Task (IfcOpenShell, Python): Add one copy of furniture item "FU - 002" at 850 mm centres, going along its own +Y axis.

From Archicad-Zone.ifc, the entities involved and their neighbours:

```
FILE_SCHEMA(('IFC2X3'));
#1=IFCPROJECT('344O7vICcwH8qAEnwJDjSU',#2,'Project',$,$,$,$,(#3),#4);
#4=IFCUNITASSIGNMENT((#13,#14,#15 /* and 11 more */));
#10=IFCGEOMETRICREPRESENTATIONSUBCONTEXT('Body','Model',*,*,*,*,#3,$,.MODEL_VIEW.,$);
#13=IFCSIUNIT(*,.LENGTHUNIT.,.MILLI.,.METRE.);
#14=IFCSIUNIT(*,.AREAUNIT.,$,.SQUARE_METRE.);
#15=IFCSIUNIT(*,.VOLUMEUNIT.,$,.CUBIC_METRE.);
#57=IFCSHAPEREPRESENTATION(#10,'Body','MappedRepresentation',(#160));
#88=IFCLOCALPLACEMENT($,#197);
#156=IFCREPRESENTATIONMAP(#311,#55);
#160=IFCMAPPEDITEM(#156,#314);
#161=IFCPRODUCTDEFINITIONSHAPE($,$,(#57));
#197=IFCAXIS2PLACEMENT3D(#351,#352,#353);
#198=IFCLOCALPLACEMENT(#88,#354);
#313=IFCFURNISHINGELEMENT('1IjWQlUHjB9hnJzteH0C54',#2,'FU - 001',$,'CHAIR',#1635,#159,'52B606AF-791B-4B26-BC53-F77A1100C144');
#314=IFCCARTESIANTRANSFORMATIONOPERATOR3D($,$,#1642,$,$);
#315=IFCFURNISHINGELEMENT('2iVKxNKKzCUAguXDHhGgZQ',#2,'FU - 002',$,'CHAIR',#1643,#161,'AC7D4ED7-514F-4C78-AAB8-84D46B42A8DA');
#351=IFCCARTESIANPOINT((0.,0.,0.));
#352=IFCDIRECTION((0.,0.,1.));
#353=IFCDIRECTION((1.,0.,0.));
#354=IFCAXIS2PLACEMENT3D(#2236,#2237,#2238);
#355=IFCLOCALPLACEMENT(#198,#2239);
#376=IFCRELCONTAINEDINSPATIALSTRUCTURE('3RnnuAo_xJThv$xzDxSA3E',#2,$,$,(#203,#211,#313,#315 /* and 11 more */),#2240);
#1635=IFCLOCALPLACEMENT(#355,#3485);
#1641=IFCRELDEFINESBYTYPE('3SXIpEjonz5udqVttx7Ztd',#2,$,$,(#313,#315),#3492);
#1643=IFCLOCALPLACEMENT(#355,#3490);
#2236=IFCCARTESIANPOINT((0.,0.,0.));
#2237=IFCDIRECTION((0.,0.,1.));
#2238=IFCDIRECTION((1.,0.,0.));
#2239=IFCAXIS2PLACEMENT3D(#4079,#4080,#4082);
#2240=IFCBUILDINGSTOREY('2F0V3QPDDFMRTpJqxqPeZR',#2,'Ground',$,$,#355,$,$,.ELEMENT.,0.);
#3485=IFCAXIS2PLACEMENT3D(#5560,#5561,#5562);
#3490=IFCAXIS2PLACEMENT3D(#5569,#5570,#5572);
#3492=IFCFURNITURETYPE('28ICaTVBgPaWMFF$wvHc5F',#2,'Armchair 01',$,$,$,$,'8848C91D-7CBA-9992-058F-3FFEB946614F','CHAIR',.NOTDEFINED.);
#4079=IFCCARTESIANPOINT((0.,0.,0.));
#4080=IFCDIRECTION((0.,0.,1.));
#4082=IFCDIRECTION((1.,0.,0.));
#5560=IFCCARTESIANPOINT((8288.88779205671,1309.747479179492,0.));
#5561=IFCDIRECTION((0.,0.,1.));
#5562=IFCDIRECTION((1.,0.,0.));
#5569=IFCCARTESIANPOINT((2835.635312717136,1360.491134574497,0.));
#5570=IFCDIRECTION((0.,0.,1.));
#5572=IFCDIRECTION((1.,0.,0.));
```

```python
import ifcopenshell
import ifcopenshell.api.geometry
import ifcopenshell.api.root
import ifcopenshell.util.element
import ifcopenshell.util.placement
import ifcopenshell.util.unit

model = ifcopenshell.open("Archicad-Zone.ifc")
unit_scale = ifcopenshell.util.unit.calculate_unit_scale(model)


def reuse_history(source, copy):
    """copy_class also copies each property set's owner history, people and application; keep the originals."""
    for rel in copy.IsDefinedBy:
        if rel.is_a("IfcRelDefinesByProperties") and (history := rel.RelatingPropertyDefinition.OwnerHistory):
            rel.RelatingPropertyDefinition.OwnerHistory = source.OwnerHistory
            ifcopenshell.util.element.remove_deep2(model, history)


source = model.by_guid("2iVKxNKKzCUAguXDHhGgZQ")
base = ifcopenshell.util.placement.get_local_placement(source.ObjectPlacement)
step = base[:3, 1] * 0.85 / unit_scale

for i in range(1, 2):
    copy = ifcopenshell.api.root.copy_class(model, product=source)
    copy.Representation = ifcopenshell.util.element.copy_deep(
        model, source.Representation, exclude=["IfcGeometricRepresentationContext", "IfcRepresentationMap"]
    )
    copy.Tag = None
    reuse_history(source, copy)
    matrix = base.copy()
    matrix[:3, 3] += i * step
    print("added at", matrix[:3, 3].round(3) + 0.0)
    ifcopenshell.api.geometry.edit_object_placement(model, product=copy, matrix=matrix, is_si=False)

model.write("Archicad-Zone-out.ifc")
```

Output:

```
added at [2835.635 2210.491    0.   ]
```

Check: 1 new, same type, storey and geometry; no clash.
